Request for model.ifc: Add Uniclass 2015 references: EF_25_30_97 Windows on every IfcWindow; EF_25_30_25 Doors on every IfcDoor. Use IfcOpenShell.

First a look at what the model holds.

```python
import ifcopenshell

model = ifcopenshell.open("model.ifc")
print(model.schema)
print("classifications:", [c.Name for c in model.by_type("IfcClassification")])
for ifc_class in ("IfcDoor", "IfcRoof", "IfcStair", "IfcWall", "IfcWindow"):
    print(ifc_class, len(model.by_type(ifc_class)))
```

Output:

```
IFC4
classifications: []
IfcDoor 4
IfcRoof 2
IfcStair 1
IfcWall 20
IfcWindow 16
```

```python
import ifcopenshell
import ifcopenshell.api.classification

model = ifcopenshell.open("model.ifc")

system = ifcopenshell.api.classification.add_classification(model, classification="Uniclass 2015")

codes = {
    "IfcWindow": ("EF_25_30_97", "Windows"),
    "IfcDoor": ("EF_25_30_25", "Doors"),
}
for ifc_class, (code, name) in codes.items():
    products = model.by_type(ifc_class)
    ifcopenshell.api.classification.add_reference(
        model, products=products, classification=system, identification=code, name=name
    )
    print(code, len(products))

model.write("model_rev.ifc")
```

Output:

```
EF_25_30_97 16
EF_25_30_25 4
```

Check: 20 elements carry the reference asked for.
